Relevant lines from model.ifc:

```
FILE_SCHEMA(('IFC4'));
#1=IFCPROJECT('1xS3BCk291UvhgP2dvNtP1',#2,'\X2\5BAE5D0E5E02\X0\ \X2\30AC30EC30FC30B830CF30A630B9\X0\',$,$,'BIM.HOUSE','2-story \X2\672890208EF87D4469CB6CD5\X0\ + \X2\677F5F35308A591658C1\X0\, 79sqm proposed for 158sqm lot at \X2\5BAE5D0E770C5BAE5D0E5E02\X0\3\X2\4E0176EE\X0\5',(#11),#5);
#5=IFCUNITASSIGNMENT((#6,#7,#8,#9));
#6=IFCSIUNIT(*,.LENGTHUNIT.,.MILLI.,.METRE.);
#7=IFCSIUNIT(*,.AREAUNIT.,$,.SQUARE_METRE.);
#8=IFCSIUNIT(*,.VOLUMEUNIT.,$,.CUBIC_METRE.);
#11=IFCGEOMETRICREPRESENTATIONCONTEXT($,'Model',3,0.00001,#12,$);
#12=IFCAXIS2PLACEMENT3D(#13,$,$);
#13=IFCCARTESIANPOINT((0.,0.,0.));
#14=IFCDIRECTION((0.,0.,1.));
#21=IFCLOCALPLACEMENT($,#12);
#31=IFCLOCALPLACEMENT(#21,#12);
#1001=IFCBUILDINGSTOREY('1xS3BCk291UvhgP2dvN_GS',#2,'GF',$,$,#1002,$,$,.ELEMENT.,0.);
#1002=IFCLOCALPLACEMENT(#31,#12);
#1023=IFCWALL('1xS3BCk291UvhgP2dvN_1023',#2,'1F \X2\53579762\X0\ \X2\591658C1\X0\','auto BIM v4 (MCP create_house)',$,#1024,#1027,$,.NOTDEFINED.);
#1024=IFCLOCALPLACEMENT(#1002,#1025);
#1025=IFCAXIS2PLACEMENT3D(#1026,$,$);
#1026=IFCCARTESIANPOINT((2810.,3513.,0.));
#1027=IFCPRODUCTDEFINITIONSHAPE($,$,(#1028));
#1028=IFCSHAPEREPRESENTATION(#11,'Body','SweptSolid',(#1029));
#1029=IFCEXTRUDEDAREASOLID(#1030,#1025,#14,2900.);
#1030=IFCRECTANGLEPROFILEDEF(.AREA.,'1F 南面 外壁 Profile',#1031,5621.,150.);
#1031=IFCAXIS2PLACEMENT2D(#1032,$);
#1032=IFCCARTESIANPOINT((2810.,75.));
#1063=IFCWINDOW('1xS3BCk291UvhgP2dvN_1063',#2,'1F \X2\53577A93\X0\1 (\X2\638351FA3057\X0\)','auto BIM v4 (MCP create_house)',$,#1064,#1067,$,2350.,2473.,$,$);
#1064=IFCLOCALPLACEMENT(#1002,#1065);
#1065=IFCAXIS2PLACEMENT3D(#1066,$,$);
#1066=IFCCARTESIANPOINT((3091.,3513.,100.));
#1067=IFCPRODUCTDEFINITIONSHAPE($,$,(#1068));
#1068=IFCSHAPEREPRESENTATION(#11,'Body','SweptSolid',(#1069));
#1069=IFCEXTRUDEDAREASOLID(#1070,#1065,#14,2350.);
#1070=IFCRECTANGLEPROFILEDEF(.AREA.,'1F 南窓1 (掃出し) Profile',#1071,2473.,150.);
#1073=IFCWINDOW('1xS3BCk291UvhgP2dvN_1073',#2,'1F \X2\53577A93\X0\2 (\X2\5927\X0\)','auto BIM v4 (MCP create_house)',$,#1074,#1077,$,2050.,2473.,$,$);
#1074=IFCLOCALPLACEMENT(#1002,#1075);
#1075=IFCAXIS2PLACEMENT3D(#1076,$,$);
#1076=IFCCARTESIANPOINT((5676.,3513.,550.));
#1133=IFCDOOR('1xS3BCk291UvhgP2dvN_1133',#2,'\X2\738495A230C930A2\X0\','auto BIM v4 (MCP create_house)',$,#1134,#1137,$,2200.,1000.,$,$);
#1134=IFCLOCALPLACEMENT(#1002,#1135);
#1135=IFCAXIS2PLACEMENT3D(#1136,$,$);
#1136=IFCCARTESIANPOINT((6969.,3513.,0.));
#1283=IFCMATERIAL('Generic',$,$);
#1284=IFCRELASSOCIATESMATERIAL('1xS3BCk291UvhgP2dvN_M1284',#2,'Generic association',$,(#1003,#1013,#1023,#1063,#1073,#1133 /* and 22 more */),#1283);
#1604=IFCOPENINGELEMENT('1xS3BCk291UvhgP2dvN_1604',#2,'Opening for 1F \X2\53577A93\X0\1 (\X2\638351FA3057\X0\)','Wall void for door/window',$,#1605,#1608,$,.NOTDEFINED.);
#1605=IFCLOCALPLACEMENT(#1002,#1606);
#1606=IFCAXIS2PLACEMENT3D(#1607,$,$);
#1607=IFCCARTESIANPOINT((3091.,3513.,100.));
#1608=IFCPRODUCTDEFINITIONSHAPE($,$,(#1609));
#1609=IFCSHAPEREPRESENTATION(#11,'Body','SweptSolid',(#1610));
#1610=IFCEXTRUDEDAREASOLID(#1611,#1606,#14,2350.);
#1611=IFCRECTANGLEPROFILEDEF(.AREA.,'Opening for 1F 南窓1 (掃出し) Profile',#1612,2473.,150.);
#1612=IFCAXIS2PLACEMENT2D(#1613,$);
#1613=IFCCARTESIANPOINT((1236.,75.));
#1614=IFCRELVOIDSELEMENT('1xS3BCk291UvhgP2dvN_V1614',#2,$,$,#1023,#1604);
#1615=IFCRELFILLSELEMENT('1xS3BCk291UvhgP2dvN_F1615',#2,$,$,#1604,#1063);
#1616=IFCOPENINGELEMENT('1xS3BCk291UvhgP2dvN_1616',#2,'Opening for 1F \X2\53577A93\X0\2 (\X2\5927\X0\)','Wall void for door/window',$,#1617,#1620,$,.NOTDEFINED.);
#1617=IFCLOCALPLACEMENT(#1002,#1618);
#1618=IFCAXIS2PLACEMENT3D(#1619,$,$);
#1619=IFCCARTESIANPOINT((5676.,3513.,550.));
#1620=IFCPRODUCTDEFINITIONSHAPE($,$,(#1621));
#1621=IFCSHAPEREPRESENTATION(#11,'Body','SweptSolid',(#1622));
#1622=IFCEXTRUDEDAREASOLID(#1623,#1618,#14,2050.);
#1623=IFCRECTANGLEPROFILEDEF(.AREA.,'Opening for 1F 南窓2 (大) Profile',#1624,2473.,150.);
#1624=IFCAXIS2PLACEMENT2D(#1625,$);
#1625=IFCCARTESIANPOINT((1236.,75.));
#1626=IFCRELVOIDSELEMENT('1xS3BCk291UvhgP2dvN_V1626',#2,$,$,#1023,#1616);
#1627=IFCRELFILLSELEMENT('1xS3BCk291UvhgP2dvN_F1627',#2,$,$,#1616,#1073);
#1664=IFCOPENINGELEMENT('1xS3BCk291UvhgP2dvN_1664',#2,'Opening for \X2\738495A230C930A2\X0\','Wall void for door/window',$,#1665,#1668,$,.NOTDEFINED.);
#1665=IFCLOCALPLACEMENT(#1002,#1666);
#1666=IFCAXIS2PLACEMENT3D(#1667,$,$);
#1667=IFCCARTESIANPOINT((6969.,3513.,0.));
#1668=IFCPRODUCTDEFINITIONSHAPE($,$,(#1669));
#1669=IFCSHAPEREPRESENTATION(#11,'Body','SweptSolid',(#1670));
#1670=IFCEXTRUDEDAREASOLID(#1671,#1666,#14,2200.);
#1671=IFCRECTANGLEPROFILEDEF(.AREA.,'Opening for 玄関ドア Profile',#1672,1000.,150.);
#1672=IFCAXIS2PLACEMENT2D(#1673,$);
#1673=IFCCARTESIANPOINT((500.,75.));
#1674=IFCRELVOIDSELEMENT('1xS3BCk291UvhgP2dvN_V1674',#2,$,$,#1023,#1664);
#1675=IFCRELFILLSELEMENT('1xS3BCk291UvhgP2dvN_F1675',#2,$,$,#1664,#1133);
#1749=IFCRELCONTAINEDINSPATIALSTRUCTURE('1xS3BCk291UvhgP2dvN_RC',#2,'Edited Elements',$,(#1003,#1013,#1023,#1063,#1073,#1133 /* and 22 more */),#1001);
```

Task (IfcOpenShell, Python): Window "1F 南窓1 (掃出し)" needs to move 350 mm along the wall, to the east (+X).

```python
import ifcopenshell
import ifcopenshell.api.geometry
import ifcopenshell.util.placement
import ifcopenshell.util.unit

model = ifcopenshell.open("model.ifc")
unit_scale = ifcopenshell.util.unit.calculate_unit_scale(model)

window = model.by_id(1063)
opening = window.FillsVoids[0].RelatingOpeningElement
wall = opening.VoidsElements[0].RelatingBuildingElement

wall_matrix = ifcopenshell.util.placement.get_local_placement(wall.ObjectPlacement)
shift = wall_matrix[:3, 0] * 0.35 / unit_scale
before = ifcopenshell.util.placement.get_local_placement(window.ObjectPlacement)[:3, 3].copy()

# The window is not placed relative to its opening, so move both.
for product in (opening, window):
    matrix = ifcopenshell.util.placement.get_local_placement(product.ObjectPlacement)
    matrix[:3, 3] += shift
    ifcopenshell.api.geometry.edit_object_placement(model, product=product, matrix=matrix, is_si=False)

after = ifcopenshell.util.placement.get_local_placement(window.ObjectPlacement)[:3, 3]
print("window moved by", (after - before).round(3) + 0.0)

model.write("model_v2.ifc")
```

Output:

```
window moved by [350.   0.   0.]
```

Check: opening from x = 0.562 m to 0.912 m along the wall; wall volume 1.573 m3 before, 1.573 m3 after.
